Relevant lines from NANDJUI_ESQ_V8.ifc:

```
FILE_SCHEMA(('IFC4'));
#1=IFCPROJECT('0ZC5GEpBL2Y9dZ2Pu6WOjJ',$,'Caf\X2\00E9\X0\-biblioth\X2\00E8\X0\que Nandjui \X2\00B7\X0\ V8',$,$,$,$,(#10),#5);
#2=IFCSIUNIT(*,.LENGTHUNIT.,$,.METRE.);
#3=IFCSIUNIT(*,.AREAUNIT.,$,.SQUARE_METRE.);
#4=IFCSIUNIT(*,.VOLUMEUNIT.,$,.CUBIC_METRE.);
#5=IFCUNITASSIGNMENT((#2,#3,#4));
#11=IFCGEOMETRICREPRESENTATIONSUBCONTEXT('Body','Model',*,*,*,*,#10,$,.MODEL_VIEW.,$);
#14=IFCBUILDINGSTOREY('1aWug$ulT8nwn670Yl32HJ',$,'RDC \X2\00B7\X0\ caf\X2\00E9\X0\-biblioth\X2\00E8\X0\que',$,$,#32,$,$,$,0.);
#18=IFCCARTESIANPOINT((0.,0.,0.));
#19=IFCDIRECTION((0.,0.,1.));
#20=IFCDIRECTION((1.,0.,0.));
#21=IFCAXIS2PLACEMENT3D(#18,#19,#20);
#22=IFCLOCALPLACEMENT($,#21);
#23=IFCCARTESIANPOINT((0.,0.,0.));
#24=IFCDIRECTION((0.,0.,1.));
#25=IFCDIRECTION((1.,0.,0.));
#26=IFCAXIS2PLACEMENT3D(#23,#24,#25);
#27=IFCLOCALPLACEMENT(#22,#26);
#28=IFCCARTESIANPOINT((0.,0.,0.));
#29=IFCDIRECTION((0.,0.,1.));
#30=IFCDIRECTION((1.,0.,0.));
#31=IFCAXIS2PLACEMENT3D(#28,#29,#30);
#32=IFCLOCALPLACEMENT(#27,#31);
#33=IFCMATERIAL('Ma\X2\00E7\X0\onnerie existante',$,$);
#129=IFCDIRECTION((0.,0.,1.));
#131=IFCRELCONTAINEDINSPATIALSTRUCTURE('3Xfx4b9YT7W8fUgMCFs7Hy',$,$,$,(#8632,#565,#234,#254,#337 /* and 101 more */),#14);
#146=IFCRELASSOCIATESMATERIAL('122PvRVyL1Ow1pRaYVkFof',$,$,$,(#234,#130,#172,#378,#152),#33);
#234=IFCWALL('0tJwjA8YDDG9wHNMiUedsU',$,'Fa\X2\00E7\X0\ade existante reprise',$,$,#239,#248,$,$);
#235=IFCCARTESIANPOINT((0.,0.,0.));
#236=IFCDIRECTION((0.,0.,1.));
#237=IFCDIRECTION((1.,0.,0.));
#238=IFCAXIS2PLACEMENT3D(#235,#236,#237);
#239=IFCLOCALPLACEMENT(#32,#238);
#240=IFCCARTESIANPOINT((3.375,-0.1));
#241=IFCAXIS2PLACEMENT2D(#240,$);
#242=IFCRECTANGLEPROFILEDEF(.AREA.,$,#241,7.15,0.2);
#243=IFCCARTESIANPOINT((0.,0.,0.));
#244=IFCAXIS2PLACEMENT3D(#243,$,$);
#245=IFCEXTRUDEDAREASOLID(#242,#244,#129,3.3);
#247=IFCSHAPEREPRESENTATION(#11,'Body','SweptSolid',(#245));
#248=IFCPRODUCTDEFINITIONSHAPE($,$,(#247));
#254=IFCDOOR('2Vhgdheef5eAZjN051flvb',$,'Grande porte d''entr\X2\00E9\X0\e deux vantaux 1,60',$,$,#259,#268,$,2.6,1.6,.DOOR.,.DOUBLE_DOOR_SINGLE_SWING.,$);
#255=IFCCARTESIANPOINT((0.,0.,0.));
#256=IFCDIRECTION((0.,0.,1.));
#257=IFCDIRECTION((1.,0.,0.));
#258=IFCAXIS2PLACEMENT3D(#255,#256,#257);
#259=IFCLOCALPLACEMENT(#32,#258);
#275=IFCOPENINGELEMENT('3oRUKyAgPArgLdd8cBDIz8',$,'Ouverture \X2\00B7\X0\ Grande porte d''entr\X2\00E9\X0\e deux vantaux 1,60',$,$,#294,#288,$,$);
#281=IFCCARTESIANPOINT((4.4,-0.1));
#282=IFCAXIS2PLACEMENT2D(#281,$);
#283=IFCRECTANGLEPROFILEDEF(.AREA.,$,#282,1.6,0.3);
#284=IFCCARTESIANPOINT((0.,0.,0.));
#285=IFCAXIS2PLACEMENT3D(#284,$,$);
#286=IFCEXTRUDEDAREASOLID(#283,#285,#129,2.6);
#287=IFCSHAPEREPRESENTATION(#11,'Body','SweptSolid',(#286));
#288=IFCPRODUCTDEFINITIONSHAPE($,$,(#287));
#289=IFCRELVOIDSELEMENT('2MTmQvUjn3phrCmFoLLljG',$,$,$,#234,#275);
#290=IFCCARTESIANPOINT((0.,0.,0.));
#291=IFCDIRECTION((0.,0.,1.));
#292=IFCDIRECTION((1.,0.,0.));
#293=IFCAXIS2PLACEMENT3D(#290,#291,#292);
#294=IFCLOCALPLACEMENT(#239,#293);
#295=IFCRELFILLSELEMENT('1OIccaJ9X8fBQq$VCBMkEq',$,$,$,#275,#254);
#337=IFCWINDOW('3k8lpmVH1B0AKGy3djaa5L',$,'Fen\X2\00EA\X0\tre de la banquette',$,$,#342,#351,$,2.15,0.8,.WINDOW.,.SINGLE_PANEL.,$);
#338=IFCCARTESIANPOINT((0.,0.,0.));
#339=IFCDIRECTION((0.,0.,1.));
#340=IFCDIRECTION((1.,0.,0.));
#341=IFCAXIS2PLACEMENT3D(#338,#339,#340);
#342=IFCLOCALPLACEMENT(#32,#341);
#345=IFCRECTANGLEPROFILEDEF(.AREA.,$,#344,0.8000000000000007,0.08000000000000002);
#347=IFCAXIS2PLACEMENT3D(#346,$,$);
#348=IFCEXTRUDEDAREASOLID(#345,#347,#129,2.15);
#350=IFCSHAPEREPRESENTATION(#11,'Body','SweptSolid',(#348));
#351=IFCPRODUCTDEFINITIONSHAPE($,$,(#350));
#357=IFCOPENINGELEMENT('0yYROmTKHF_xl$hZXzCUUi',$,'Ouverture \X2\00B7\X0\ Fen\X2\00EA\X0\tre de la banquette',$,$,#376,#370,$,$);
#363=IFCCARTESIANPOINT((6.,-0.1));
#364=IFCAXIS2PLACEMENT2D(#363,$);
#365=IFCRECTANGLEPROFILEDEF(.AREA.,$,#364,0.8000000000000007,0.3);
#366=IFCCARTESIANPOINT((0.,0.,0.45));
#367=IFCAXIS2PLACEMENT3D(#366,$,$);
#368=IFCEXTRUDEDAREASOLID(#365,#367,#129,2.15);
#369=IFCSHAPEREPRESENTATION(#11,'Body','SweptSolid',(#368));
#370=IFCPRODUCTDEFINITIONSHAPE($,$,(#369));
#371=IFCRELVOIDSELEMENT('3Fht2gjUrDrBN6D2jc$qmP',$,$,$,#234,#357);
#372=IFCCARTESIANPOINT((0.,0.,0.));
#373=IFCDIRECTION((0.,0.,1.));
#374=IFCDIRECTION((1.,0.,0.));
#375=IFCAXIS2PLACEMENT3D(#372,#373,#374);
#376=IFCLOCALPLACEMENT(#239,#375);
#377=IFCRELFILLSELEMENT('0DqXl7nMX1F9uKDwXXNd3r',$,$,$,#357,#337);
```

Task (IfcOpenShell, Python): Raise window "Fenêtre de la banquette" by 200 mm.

```python
import numpy as np
import ifcopenshell
import ifcopenshell.api.geometry
import ifcopenshell.util.placement
import ifcopenshell.util.unit

model = ifcopenshell.open("NANDJUI_ESQ_V8.ifc")
unit_scale = ifcopenshell.util.unit.calculate_unit_scale(model)

window = model.by_guid("3k8lpmVH1B0AKGy3djaa5L")
opening = window.FillsVoids[0].RelatingOpeningElement
dz = 0.2 / unit_scale

shift = np.array([0.0, 0.0, dz])
# The window is not placed relative to its opening, so move both.
for product in (opening, window):
    matrix = ifcopenshell.util.placement.get_local_placement(product.ObjectPlacement)
    matrix[:3, 3] += shift
    ifcopenshell.api.geometry.edit_object_placement(model, product=product, matrix=matrix, is_si=False)

print(f"moved by {dz * unit_scale:+.3f} m")

model.write("NANDJUI_ESQ_V8_v2.ifc")
```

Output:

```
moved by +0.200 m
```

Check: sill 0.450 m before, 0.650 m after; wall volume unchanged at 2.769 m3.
